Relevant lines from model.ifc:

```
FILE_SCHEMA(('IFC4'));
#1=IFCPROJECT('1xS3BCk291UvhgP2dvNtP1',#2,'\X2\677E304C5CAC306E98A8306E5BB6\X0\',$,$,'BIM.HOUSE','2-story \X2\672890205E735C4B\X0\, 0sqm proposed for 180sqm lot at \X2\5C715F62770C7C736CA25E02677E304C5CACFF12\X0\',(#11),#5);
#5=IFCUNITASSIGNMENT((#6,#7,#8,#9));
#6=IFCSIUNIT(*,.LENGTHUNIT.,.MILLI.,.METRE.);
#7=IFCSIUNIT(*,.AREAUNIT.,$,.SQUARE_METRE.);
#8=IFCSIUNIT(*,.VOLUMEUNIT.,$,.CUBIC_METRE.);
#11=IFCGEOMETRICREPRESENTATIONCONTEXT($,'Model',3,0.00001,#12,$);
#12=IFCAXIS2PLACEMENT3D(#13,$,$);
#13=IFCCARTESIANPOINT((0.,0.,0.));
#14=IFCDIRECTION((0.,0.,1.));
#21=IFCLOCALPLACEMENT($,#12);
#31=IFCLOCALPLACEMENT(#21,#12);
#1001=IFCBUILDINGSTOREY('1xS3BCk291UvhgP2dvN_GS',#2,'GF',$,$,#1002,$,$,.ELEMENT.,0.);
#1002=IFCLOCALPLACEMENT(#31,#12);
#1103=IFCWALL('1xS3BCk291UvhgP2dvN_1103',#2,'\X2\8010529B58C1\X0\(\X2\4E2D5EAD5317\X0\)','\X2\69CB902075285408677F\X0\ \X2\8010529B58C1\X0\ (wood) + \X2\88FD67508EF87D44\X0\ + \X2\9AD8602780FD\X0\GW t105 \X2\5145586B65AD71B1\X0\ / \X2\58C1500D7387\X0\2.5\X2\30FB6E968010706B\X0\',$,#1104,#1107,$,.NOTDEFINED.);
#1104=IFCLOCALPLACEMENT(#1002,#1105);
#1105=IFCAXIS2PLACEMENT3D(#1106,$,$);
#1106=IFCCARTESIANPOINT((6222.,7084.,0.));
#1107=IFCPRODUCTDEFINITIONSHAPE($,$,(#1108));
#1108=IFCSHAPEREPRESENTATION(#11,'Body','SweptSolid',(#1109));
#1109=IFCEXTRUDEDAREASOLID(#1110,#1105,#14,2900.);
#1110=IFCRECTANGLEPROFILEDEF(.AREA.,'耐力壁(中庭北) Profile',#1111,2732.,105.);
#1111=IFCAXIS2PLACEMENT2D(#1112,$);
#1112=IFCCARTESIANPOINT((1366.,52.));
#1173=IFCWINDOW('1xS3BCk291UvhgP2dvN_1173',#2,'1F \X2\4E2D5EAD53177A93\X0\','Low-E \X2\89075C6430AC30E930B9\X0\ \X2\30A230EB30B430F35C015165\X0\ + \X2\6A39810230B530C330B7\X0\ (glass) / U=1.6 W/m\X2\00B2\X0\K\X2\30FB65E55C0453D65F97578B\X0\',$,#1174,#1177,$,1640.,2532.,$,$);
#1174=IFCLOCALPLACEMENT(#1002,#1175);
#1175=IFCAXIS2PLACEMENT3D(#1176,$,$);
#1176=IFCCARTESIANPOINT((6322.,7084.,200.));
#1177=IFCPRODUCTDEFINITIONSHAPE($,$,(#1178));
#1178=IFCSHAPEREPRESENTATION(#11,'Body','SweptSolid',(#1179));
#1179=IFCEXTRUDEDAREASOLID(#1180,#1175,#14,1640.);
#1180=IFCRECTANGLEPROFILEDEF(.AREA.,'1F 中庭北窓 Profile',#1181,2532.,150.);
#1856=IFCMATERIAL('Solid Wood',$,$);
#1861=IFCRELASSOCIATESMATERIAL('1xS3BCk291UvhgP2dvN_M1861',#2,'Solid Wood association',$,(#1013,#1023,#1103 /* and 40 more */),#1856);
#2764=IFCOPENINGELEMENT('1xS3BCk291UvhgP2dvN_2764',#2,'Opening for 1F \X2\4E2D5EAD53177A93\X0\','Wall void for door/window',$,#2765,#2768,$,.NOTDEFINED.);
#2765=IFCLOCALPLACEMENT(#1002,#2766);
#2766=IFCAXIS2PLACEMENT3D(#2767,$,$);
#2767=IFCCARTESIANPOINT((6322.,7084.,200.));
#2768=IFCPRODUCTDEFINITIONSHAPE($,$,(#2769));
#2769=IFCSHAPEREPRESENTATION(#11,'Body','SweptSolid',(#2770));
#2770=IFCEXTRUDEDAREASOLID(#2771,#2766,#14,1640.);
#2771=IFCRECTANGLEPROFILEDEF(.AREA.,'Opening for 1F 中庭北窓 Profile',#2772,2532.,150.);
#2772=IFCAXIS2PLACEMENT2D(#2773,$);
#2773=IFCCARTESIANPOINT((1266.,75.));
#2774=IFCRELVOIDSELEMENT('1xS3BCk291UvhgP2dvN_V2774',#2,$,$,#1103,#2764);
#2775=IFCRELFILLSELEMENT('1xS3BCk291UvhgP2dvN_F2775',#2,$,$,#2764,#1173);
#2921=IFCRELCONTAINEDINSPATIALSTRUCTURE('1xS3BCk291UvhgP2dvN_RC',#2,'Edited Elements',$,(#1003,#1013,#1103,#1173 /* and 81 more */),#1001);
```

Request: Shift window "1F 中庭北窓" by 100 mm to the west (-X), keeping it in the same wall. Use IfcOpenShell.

```python
import ifcopenshell
import ifcopenshell.api.geometry
import ifcopenshell.util.placement
import ifcopenshell.util.unit

model = ifcopenshell.open("model.ifc")
unit_scale = ifcopenshell.util.unit.calculate_unit_scale(model)

window = model.by_guid("1xS3BCk291UvhgP2dvN_1173")
opening = window.FillsVoids[0].RelatingOpeningElement
wall = opening.VoidsElements[0].RelatingBuildingElement

wall_matrix = ifcopenshell.util.placement.get_local_placement(wall.ObjectPlacement)
shift = wall_matrix[:3, 0] * -0.1 / unit_scale
before = ifcopenshell.util.placement.get_local_placement(window.ObjectPlacement)[:3, 3].copy()

# The window is not placed relative to its opening, so move both.
for product in (opening, window):
    matrix = ifcopenshell.util.placement.get_local_placement(product.ObjectPlacement)
    matrix[:3, 3] += shift
    ifcopenshell.api.geometry.edit_object_placement(model, product=product, matrix=matrix, is_si=False)

after = ifcopenshell.util.placement.get_local_placement(window.ObjectPlacement)[:3, 3]
print("window moved by", (after - before).round(3) + 0.0)

model.write("model-out.ifc")
```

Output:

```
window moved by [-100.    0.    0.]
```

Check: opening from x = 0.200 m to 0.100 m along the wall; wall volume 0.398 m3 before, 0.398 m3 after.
